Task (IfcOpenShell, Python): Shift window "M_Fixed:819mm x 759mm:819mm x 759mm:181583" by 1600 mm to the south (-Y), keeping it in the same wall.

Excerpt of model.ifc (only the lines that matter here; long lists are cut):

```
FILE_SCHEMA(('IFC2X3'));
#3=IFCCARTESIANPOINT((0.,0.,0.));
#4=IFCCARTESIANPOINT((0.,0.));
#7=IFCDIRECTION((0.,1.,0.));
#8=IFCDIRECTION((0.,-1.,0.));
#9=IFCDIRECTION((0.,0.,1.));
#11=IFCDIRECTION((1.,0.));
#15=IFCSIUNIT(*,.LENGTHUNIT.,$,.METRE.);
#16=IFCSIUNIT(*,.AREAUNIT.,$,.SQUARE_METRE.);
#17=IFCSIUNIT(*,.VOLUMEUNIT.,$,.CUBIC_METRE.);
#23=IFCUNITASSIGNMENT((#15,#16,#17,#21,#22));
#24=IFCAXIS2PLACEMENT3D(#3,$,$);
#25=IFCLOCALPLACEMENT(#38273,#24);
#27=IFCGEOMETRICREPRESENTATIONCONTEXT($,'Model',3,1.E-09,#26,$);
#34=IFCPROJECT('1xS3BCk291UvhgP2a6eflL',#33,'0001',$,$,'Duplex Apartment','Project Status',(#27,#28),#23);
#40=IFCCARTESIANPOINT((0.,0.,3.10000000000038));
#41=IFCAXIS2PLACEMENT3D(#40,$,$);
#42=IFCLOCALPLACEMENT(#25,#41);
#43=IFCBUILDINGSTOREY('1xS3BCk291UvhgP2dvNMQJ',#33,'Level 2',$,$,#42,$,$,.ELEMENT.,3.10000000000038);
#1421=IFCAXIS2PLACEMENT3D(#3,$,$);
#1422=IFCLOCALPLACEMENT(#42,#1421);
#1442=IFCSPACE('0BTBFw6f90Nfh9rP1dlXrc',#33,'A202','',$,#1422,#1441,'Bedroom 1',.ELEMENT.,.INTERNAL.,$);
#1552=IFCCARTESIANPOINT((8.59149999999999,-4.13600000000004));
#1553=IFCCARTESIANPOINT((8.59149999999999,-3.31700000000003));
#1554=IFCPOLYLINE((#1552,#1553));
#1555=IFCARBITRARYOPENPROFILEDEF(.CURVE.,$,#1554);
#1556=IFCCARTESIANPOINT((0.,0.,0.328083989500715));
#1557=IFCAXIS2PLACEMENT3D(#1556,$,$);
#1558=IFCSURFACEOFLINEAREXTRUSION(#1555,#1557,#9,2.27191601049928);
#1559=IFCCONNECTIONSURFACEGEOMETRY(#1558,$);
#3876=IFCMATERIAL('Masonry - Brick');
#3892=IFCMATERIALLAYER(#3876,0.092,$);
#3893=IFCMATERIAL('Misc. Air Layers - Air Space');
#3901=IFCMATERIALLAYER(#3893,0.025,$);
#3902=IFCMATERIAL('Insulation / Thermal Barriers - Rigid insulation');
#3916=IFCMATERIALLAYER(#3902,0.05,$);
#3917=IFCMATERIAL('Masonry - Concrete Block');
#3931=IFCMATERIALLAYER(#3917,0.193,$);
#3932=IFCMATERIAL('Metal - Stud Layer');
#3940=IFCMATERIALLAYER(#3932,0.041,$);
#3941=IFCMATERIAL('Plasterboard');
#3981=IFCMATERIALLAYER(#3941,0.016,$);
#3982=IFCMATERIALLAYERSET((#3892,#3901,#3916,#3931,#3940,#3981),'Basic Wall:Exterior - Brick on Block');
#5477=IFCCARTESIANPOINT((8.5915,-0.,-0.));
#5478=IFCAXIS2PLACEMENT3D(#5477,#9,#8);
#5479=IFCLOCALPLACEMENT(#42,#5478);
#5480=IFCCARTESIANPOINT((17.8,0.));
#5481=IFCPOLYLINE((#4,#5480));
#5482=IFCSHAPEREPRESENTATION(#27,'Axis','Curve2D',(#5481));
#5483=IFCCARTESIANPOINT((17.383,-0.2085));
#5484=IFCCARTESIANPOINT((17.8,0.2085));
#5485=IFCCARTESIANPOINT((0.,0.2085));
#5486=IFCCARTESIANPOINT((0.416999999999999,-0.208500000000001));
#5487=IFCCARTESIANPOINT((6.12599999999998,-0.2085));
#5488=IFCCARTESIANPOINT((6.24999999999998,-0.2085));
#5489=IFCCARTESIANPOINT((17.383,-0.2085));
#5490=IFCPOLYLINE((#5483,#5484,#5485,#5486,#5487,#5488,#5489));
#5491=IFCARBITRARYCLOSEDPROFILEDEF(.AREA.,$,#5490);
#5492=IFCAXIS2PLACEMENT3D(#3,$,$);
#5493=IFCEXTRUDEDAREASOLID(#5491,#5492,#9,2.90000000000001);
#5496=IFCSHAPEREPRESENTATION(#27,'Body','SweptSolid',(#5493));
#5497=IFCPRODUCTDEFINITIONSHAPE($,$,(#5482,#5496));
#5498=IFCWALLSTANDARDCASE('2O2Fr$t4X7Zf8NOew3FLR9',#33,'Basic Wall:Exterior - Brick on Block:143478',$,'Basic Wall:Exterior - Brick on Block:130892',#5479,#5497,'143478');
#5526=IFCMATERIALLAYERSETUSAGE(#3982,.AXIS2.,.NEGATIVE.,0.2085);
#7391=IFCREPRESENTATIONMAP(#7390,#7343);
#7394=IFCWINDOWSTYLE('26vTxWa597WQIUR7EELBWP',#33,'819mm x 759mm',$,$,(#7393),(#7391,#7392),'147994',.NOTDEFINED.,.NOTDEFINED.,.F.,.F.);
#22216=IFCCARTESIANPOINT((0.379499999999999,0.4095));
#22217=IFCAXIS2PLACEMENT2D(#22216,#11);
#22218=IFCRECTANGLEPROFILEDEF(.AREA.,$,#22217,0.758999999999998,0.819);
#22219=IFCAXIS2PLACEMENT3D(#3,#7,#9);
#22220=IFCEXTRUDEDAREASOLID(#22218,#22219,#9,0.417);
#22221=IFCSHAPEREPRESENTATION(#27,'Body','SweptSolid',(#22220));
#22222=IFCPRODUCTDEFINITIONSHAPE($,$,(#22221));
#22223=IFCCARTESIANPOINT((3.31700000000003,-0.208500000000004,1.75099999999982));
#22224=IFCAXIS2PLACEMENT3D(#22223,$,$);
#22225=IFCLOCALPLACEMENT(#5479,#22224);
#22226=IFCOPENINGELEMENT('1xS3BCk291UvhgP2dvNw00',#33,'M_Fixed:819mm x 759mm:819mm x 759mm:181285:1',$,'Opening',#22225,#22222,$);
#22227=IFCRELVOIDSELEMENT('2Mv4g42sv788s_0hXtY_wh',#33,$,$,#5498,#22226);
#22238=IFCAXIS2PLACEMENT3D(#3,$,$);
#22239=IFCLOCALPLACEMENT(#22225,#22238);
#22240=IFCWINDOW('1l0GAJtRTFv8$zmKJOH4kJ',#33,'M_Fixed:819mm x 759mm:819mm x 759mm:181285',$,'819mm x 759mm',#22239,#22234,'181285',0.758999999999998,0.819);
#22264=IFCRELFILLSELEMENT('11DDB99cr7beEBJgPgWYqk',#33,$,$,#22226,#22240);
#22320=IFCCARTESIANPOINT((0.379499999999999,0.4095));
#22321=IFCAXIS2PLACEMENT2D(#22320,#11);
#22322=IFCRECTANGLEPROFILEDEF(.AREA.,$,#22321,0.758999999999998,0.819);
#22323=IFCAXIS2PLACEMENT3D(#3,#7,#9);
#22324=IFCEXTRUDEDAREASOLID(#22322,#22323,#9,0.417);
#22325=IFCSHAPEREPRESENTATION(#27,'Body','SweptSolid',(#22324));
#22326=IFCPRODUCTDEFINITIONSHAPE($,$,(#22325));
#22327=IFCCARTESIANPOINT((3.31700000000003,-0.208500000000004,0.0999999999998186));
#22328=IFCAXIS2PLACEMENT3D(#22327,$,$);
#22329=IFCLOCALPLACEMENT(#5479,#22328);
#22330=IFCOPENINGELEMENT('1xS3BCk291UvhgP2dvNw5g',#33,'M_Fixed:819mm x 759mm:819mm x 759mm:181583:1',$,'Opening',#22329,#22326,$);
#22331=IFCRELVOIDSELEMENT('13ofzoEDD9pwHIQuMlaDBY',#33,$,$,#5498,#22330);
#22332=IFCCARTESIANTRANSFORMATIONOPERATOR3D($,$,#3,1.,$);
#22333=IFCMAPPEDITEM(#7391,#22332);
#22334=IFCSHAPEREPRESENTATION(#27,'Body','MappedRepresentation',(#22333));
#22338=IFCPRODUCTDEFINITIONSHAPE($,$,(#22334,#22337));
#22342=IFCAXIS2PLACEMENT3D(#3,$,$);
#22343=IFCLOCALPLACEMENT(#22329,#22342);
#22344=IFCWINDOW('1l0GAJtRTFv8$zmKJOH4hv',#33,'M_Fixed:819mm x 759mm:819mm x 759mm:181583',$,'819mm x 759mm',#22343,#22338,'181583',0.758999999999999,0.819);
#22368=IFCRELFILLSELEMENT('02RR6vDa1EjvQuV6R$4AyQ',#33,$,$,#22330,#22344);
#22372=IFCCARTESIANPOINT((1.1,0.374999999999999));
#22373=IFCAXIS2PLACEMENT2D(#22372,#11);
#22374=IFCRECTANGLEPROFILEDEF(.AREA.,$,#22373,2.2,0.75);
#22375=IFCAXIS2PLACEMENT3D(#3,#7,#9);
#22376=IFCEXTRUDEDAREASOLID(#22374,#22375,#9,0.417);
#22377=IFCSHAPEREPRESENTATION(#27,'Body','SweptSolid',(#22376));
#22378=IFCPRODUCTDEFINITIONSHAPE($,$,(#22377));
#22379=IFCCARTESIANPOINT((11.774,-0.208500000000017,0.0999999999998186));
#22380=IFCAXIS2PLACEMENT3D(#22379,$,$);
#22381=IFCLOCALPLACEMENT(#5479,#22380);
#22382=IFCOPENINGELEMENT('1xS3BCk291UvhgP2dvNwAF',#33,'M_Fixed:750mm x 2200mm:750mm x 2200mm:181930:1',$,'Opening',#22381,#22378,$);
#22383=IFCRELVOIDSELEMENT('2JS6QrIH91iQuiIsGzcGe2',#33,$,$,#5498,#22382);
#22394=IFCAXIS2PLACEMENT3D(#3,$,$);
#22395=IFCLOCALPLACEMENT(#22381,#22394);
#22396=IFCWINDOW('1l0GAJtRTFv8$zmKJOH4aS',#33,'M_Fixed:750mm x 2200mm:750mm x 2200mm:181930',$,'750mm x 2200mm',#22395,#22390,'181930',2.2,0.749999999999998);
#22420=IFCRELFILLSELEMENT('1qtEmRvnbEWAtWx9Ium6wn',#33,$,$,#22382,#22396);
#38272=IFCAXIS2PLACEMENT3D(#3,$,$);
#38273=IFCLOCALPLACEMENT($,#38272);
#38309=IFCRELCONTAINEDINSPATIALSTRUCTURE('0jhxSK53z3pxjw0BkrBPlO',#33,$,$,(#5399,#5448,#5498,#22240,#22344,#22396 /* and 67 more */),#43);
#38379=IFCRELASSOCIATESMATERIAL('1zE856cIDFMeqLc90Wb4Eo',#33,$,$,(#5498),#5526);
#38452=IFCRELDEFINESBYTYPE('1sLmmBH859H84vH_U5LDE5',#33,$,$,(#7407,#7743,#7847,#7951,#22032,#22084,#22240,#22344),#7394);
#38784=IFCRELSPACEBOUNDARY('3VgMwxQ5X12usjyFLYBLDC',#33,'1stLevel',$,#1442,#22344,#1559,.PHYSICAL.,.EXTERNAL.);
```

```python
import numpy as np
import ifcopenshell
import ifcopenshell.api.geometry
import ifcopenshell.util.placement

model = ifcopenshell.open("model.ifc")

window = model.by_guid("1l0GAJtRTFv8$zmKJOH4hv")
opening = window.FillsVoids[0].RelatingOpeningElement
wall = opening.VoidsElements[0].RelatingBuildingElement

wall_matrix = ifcopenshell.util.placement.get_local_placement(wall.ObjectPlacement)
shift = wall_matrix[:3, 0] * 1.6
before = ifcopenshell.util.placement.get_local_placement(window.ObjectPlacement)[:3, 3].copy()

# The window is placed relative to its opening, so it follows when the opening moves.
matrix = ifcopenshell.util.placement.get_local_placement(opening.ObjectPlacement)
matrix[:3, 3] += shift
ifcopenshell.api.geometry.edit_object_placement(
    model, product=opening, matrix=matrix, is_si=False, should_transform_children=True
)

# Space boundary surfaces are stored in each space's coordinates; move them too.
for rel in window.ProvidesBoundaries:
    if not rel.ConnectionGeometry:
        continue
    surface = rel.ConnectionGeometry.SurfaceOnRelatingElement
    space_matrix = ifcopenshell.util.placement.get_local_placement(rel.RelatingSpace.ObjectPlacement)
    point = np.array(surface.Position.Location.Coordinates) + space_matrix[:3, :3].T @ shift
    surface.Position = model.createIfcAxis2Placement3D(
        model.createIfcCartesianPoint(point.tolist()), surface.Position.Axis, surface.Position.RefDirection
    )

after = ifcopenshell.util.placement.get_local_placement(window.ObjectPlacement)[:3, 3]
print("window moved by", (after - before).round(3) + 0.0)

model.write("model_v2.ifc")
```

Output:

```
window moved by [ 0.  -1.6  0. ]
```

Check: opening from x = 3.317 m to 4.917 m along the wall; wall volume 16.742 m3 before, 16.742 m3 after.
